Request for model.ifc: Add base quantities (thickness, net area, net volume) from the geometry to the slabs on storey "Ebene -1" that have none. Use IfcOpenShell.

First a look at what the model holds.

```python
import ifcopenshell
import ifcopenshell.util.element
import ifcopenshell.util.unit

model = ifcopenshell.open("model.ifc")
print(model.schema)
for unit_type in ("LENGTHUNIT", "AREAUNIT", "VOLUMEUNIT"):
    print(unit_type, ifcopenshell.util.unit.calculate_unit_scale(model, unit_type))
storey = next(s for s in model.by_type("IfcBuildingStorey") if s.Name == "Ebene -1")
slabs = [e for e in ifcopenshell.util.element.get_decomposition(storey) if e.is_a("IfcSlab")]
for e in sorted(slabs, key=lambda e: e.id()):
    print(e.id(), e.is_a(), e.Name, list(ifcopenshell.util.element.get_psets(e, qtos_only=True)), sep=" | ")
```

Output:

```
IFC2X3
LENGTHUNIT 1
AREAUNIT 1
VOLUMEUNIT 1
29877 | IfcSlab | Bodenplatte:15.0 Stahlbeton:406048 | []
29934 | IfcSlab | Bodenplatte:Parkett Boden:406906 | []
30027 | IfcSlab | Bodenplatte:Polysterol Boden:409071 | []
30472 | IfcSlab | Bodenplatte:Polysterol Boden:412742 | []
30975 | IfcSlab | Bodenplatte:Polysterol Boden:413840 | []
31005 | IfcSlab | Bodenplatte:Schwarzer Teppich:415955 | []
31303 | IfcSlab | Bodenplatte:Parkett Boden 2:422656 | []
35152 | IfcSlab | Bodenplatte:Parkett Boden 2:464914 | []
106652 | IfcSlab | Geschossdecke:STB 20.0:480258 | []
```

```python
import ifcopenshell
import ifcopenshell.api.pset
import ifcopenshell.geom
import ifcopenshell.util.element
import ifcopenshell.util.shape
import ifcopenshell.util.unit

model = ifcopenshell.open("model.ifc")
unit_scale = ifcopenshell.util.unit.calculate_unit_scale(model)
area_scale = ifcopenshell.util.unit.calculate_unit_scale(model, "AREAUNIT")
volume_scale = ifcopenshell.util.unit.calculate_unit_scale(model, "VOLUMEUNIT")
settings = ifcopenshell.geom.settings()

storey = next(s for s in model.by_type("IfcBuildingStorey") if s.Name == "Ebene -1")
slabs = [e for e in ifcopenshell.util.element.get_decomposition(storey) if e.is_a("IfcSlab")]

for e in sorted(slabs, key=lambda e: e.id()):
    if ifcopenshell.util.element.get_psets(e, qtos_only=True, should_inherit=False):
        continue
    # Geometry comes back in metres, in the element's own axes.
    shape = ifcopenshell.geom.create_shape(settings, e)
    values = {
        "Width": ifcopenshell.util.shape.get_z(shape.geometry) / unit_scale,
        "NetArea": ifcopenshell.util.shape.get_footprint_area(shape.geometry) / area_scale,
        "NetVolume": ifcopenshell.util.shape.get_volume(shape.geometry) / volume_scale,
    }
    qto = ifcopenshell.api.pset.add_qto(model, product=e, name="BaseQuantities")
    ifcopenshell.api.pset.edit_qto(model, qto=qto, properties=values)
    print(e.id(), {k: round(v, 3) for k, v in values.items()})

model.write("model_v2.ifc")
```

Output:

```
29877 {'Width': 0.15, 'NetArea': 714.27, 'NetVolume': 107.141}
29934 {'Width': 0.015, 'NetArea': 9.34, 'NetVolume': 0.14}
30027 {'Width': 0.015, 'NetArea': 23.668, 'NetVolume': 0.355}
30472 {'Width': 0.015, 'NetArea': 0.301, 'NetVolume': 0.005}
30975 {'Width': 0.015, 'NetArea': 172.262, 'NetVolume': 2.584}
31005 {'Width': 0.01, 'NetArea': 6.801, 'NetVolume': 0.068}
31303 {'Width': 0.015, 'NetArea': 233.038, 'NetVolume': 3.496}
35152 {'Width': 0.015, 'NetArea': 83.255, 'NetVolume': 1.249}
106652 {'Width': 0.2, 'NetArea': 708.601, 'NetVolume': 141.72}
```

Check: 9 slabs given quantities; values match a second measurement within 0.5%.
